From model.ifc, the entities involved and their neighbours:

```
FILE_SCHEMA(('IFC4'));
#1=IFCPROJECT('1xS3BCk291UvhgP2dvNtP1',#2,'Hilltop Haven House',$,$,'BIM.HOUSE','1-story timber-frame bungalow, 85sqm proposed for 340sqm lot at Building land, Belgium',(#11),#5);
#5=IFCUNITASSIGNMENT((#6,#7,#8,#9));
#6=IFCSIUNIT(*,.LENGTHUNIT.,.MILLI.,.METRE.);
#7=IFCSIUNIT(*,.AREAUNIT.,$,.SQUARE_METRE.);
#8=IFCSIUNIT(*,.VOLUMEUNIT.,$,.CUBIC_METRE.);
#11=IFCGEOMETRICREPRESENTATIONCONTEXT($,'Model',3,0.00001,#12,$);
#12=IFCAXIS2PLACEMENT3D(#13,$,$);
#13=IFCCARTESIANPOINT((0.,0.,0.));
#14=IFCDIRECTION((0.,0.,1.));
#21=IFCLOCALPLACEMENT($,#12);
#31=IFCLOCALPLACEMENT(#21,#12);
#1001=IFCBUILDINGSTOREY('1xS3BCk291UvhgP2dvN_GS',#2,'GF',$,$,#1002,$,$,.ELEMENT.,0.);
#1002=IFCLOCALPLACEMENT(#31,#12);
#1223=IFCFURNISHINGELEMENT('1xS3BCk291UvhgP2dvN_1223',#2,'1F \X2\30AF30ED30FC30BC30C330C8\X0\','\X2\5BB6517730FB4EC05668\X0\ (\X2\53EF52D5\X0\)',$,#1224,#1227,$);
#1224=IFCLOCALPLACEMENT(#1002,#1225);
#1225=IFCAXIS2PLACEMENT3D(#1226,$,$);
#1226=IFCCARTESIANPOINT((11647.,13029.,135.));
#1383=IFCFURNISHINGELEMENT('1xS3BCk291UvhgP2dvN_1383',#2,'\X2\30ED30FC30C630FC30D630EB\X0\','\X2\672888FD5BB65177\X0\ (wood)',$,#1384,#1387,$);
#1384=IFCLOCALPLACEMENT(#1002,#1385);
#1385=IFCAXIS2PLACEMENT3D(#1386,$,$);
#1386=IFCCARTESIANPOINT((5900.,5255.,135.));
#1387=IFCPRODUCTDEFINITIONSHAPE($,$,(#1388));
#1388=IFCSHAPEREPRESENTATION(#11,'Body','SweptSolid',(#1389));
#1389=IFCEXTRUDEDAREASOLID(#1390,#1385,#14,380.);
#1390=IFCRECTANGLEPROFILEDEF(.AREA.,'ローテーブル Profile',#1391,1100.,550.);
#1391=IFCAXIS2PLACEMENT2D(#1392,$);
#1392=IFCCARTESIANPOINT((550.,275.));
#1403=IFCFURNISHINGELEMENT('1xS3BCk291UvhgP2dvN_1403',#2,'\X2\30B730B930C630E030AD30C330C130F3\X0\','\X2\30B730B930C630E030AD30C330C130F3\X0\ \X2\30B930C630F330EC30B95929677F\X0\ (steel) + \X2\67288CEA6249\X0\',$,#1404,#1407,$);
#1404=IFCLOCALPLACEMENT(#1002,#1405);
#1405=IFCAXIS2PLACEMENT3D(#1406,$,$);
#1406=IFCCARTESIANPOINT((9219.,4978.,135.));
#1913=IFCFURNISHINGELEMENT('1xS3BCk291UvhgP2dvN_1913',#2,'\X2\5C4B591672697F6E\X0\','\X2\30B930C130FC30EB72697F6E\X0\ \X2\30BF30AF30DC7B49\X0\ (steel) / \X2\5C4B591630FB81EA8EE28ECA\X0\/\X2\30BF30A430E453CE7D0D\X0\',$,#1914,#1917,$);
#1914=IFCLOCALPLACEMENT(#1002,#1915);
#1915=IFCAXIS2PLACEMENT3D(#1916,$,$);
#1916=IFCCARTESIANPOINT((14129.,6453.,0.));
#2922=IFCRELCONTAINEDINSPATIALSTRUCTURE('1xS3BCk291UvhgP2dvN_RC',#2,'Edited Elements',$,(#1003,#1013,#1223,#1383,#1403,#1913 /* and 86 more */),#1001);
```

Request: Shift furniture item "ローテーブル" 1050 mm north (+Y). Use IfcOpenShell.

```python
import ifcopenshell
import ifcopenshell.api.geometry
import ifcopenshell.util.placement

model = ifcopenshell.open("model.ifc")

item = model.by_id(1383)
matrix = ifcopenshell.util.placement.get_local_placement(item.ObjectPlacement)
matrix[1, 3] += 1050.0
ifcopenshell.api.geometry.edit_object_placement(model, product=item, matrix=matrix, is_si=False)

print(ifcopenshell.util.placement.get_local_placement(item.ObjectPlacement).round(3) + 0.0)

model.write("model_updated.ifc")
```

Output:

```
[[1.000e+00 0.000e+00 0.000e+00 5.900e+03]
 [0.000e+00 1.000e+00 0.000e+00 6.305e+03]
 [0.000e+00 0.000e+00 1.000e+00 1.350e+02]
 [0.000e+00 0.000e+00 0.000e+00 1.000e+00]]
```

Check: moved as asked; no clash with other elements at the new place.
